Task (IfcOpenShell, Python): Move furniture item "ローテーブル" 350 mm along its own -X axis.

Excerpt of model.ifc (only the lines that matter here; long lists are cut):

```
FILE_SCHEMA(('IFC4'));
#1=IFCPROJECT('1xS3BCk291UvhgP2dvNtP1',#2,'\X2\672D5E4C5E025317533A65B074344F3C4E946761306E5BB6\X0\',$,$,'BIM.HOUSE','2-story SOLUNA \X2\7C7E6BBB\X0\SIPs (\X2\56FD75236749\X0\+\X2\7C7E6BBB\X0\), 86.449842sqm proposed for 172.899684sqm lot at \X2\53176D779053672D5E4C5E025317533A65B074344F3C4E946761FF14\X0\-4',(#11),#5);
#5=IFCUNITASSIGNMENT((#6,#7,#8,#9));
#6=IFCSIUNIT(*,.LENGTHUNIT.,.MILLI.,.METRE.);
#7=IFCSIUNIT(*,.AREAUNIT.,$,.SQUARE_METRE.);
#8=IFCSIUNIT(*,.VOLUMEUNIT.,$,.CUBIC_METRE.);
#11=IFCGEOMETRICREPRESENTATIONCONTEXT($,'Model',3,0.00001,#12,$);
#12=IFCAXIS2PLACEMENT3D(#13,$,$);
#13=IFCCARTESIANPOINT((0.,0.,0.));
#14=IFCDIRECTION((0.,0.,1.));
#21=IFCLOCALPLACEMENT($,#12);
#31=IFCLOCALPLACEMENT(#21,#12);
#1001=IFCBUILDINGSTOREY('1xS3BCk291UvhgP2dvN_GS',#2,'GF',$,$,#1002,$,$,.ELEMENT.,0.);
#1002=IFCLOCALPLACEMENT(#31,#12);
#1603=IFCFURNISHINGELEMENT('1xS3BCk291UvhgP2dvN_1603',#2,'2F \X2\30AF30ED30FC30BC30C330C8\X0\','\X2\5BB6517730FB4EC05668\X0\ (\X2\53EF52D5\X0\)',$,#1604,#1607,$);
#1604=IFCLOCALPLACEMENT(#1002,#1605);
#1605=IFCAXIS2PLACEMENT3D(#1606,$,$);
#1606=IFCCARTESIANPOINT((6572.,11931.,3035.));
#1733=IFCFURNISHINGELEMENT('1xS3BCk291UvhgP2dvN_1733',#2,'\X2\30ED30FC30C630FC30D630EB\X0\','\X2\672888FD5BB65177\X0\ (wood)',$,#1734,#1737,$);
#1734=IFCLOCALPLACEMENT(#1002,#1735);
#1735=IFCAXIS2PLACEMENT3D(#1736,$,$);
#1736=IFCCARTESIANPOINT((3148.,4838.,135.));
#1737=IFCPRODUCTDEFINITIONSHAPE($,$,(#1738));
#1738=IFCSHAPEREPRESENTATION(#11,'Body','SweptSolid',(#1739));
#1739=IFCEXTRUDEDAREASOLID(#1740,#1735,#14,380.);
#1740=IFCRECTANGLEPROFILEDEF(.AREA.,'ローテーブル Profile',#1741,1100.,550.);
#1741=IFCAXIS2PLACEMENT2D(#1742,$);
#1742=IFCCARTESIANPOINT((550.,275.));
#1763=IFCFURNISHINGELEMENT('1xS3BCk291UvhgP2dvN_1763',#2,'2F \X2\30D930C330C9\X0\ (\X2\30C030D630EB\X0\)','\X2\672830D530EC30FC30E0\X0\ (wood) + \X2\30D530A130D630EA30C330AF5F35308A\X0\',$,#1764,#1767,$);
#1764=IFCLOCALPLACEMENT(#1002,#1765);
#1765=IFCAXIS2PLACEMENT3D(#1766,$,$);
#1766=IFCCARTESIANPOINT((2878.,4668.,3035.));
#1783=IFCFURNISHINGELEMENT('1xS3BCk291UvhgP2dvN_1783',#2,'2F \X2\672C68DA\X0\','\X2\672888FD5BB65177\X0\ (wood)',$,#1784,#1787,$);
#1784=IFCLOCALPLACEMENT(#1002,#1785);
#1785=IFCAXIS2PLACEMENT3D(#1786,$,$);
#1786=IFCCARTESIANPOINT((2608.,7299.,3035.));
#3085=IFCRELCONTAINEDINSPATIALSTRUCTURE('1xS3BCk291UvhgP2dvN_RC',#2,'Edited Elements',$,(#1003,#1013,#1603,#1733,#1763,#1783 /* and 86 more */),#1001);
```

```python
import ifcopenshell
import ifcopenshell.api.geometry
import ifcopenshell.util.placement
import ifcopenshell.util.unit

model = ifcopenshell.open("model.ifc")
unit_scale = ifcopenshell.util.unit.calculate_unit_scale(model)

item = model.by_guid("1xS3BCk291UvhgP2dvN_1733")
matrix = ifcopenshell.util.placement.get_local_placement(item.ObjectPlacement)
matrix[:3, 3] -= matrix[:3, 0] * 0.35 / unit_scale
ifcopenshell.api.geometry.edit_object_placement(model, product=item, matrix=matrix, is_si=False)

print(ifcopenshell.util.placement.get_local_placement(item.ObjectPlacement).round(3) + 0.0)

model.write("model_rev.ifc")
```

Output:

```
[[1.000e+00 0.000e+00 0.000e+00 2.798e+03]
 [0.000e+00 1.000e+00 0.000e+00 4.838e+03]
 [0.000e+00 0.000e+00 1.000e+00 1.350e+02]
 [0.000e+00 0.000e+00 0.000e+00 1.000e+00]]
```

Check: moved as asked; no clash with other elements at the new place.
